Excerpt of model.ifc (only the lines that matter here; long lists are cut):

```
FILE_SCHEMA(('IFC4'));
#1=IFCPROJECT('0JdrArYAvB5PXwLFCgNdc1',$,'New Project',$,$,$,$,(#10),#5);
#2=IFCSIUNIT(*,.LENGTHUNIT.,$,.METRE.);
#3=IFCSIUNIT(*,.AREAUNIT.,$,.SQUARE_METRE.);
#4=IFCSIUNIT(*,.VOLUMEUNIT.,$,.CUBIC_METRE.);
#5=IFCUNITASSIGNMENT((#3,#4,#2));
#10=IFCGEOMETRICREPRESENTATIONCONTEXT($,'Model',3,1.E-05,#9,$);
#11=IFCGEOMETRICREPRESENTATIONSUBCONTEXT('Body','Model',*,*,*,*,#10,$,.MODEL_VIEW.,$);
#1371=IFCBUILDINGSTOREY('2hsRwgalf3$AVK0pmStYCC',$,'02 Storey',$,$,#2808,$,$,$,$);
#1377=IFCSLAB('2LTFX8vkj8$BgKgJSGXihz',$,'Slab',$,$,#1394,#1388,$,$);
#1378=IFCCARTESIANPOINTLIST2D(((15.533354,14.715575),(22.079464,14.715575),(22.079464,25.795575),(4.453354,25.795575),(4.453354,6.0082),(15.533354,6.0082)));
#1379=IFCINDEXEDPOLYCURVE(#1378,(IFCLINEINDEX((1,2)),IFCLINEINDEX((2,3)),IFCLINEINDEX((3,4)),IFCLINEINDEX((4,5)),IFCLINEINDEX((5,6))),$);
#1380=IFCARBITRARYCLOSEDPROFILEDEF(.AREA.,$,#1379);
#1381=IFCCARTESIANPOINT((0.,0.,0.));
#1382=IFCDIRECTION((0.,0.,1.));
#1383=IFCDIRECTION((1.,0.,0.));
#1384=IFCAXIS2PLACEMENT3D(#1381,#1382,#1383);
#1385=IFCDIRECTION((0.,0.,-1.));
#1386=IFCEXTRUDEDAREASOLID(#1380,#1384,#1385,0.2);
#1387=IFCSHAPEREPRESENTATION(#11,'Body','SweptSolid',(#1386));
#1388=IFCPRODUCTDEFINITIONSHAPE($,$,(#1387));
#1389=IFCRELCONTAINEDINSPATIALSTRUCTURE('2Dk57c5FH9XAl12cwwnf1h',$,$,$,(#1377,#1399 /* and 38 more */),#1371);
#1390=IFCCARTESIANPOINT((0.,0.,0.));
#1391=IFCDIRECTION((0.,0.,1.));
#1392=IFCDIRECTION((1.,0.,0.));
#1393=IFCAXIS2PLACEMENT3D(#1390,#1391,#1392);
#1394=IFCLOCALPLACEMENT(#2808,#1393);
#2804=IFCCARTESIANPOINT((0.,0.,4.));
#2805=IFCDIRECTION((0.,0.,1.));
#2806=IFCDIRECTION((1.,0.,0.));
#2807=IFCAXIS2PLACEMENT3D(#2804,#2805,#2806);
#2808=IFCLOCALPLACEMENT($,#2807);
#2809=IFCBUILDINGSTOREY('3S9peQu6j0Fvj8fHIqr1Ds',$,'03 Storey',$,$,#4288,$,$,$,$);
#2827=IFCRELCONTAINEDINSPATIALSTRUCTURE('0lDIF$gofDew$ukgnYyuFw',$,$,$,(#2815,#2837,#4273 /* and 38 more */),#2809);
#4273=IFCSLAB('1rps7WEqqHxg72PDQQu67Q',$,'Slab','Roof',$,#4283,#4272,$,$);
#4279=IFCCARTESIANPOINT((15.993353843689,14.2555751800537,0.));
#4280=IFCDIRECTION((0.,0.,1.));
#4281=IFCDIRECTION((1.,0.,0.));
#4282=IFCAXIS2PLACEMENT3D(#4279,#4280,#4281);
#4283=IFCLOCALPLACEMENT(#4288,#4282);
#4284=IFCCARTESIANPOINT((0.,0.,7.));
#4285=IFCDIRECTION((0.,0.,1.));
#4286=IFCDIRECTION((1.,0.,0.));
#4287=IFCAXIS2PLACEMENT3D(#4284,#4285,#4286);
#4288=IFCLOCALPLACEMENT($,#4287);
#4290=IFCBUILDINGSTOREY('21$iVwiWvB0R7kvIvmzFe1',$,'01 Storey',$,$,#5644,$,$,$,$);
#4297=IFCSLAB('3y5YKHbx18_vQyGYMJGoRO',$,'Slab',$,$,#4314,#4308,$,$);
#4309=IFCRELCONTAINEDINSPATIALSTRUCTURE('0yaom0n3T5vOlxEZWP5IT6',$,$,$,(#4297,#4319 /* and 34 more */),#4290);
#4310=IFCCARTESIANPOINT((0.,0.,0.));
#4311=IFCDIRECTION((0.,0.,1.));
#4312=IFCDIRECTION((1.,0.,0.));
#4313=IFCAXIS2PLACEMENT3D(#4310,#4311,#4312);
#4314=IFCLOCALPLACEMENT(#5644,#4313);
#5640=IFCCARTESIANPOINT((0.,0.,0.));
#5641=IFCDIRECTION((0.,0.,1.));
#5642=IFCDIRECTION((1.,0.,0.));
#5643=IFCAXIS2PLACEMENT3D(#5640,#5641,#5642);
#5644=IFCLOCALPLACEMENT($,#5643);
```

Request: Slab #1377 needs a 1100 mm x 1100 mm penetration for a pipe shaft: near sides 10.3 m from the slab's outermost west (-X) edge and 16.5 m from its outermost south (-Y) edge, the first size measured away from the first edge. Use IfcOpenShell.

```python
import numpy as np
import ifcopenshell
import ifcopenshell.api.feature
import ifcopenshell.api.geometry
import ifcopenshell.api.root
import ifcopenshell.geom
import ifcopenshell.util.placement
import ifcopenshell.util.representation
import ifcopenshell.util.shape
import ifcopenshell.util.unit

model = ifcopenshell.open("model.ifc")
unit_scale = ifcopenshell.util.unit.calculate_unit_scale(model)
settings = ifcopenshell.geom.settings()


def volume(element):
    """Net volume in cubic metres, openings subtracted."""
    shape = ifcopenshell.geom.create_shape(settings, element)
    return ifcopenshell.util.shape.get_volume(shape.geometry)


slab = model.by_id(1377)
before = volume(slab)

# Extent in the slab's own axes, in metres. The edges named are its -X and -Y sides.
slab_shape = ifcopenshell.geom.create_shape(settings, slab)
vertices = ifcopenshell.util.shape.get_vertices(slab_shape.geometry)
x_min, y_min, bottom = vertices.min(axis=0)
top = vertices[:, 2].max()

opening = ifcopenshell.api.root.create_entity(model, ifc_class="IfcOpeningElement", name="Pipe shaft opening", predefined_type="OPENING")
context = ifcopenshell.util.representation.get_context(model, "Model", "Body", "MODEL_VIEW")
width, depth = 1.1, 1.1
outline = [(0.0, 0.0), (width, 0.0), (width, depth), (0.0, depth), (0.0, 0.0)]
# Overshoot both faces by 50 mm so the cut is clean.
shape = ifcopenshell.api.geometry.add_slab_representation(
    model, context=context, depth=top - bottom + 0.1, polyline=outline
)
ifcopenshell.api.geometry.assign_representation(model, product=opening, representation=shape)

matrix = ifcopenshell.util.placement.get_local_placement(slab.ObjectPlacement)
matrix[:, 3] = matrix @ np.append(np.array([x_min + 10.3, y_min + 16.5, bottom - 0.05]) / unit_scale, 1.0)
ifcopenshell.api.geometry.edit_object_placement(model, product=opening, matrix=matrix, is_si=False)
ifcopenshell.api.feature.add_feature(model, feature=opening, element=slab)

after = volume(slab)

print(f"slab volume {before:.3f} -> {after:.3f} m3")

model.write("model_v2.ifc")
```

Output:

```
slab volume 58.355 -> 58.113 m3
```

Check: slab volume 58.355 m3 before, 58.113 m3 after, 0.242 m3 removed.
